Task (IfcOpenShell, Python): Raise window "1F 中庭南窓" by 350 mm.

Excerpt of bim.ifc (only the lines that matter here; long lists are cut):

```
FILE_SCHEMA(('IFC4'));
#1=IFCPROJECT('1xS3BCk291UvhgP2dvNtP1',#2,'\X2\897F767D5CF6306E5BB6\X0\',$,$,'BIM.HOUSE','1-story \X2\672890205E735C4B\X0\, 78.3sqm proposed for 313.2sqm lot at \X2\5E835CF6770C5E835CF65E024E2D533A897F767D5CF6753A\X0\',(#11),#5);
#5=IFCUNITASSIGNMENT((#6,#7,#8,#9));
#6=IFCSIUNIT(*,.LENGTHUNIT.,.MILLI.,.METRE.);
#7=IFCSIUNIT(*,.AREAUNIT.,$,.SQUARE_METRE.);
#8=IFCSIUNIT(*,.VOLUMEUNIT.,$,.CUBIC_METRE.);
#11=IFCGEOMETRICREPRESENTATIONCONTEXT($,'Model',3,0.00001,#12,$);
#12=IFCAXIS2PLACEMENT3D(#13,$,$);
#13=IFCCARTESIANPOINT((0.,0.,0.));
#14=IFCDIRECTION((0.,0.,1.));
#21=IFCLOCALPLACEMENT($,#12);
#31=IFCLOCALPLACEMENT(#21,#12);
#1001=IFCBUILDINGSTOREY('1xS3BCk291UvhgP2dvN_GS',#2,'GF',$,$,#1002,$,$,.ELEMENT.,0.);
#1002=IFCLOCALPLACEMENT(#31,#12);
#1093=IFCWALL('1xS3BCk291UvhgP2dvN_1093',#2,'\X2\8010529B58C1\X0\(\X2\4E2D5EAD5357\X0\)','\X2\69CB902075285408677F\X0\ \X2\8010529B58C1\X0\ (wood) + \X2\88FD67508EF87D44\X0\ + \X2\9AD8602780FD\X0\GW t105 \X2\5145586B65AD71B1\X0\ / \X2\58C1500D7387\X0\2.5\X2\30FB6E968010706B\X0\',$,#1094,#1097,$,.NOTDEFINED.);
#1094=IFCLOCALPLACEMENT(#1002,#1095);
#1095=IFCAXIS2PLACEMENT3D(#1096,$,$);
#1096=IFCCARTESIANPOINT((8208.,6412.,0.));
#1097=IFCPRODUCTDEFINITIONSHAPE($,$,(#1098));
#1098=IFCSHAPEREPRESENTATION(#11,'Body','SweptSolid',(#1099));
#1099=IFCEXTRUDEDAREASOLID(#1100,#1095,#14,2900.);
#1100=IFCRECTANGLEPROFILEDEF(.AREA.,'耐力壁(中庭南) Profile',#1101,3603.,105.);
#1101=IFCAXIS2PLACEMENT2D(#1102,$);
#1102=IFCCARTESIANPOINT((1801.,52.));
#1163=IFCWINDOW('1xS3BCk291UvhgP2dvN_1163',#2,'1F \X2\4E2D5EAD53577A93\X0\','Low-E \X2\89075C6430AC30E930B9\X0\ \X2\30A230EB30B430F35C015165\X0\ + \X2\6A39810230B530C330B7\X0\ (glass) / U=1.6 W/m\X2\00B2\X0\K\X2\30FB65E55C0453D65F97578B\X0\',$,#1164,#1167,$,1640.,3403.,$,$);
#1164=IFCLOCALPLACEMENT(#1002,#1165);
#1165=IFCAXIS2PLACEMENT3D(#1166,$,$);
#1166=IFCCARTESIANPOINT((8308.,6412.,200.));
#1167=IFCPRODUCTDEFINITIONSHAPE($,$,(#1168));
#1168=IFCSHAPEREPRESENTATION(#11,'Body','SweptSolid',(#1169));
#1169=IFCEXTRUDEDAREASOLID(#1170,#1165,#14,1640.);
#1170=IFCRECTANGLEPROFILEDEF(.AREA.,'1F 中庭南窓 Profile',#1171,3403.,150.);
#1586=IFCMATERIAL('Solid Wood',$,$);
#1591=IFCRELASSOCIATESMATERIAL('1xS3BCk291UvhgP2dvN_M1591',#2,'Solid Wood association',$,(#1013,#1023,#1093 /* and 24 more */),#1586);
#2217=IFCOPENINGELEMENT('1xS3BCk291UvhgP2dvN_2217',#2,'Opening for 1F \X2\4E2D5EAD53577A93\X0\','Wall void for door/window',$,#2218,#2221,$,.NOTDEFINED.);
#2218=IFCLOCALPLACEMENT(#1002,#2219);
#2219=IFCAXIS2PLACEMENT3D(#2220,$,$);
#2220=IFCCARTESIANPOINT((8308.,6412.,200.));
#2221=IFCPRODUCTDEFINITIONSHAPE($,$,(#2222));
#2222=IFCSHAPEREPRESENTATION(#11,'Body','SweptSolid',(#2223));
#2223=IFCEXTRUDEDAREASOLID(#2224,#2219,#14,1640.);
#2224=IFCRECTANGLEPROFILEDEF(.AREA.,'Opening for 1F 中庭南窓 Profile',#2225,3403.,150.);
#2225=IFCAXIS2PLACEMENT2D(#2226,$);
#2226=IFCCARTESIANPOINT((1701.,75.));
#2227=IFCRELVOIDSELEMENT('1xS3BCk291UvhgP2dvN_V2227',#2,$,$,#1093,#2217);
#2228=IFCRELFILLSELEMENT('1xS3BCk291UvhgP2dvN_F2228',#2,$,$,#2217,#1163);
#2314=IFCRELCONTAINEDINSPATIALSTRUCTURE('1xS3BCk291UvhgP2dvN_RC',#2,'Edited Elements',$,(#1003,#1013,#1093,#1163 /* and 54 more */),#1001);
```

```python
import numpy as np
import ifcopenshell
import ifcopenshell.api.geometry
import ifcopenshell.util.placement
import ifcopenshell.util.unit

model = ifcopenshell.open("bim.ifc")
unit_scale = ifcopenshell.util.unit.calculate_unit_scale(model)

window = model.by_guid("1xS3BCk291UvhgP2dvN_1163")
opening = window.FillsVoids[0].RelatingOpeningElement
dz = 350.0

shift = np.array([0.0, 0.0, dz])
# The window is not placed relative to its opening, so move both.
for product in (opening, window):
    matrix = ifcopenshell.util.placement.get_local_placement(product.ObjectPlacement)
    matrix[:3, 3] += shift
    ifcopenshell.api.geometry.edit_object_placement(model, product=product, matrix=matrix, is_si=False)

print(f"moved by {dz * unit_scale:+.3f} m")

model.write("bim_rev.ifc")
```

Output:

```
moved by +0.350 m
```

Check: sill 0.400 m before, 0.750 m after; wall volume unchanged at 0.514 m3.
